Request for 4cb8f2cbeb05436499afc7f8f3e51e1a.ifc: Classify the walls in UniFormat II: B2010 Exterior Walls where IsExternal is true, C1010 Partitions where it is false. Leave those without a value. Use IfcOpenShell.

First a look at what the model holds.

```python
import ifcopenshell
import ifcopenshell.util.element

model = ifcopenshell.open("4cb8f2cbeb05436499afc7f8f3e51e1a.ifc")
print(model.schema)
print("classifications:", [c.Name for c in model.by_type("IfcClassification")])
values = [ifcopenshell.util.element.get_pset(e, "Pset_WallCommon", "IsExternal") for e in model.by_type("IfcWall")]
for value in (True, False, None):
    print("IsExternal", value, values.count(value))
```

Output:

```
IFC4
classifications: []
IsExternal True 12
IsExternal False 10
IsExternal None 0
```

```python
import ifcopenshell
import ifcopenshell.api.classification
import ifcopenshell.util.element

model = ifcopenshell.open("4cb8f2cbeb05436499afc7f8f3e51e1a.ifc")

system = ifcopenshell.api.classification.add_classification(model, classification="UniFormat II")

walls = model.by_type("IfcWall")
external = {e: ifcopenshell.util.element.get_pset(e, "Pset_WallCommon", "IsExternal") for e in walls}
for flag, code, name in ((True, "B2010", "Exterior Walls"), (False, "C1010", "Partitions")):
    products = [e for e in walls if external[e] is flag]
    ifcopenshell.api.classification.add_reference(
        model, products=products, classification=system, identification=code, name=name
    )
    print(code, len(products))

model.write("4cb8f2cbeb05436499afc7f8f3e51e1a_updated.ifc")
```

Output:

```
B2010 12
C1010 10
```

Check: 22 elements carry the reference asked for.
